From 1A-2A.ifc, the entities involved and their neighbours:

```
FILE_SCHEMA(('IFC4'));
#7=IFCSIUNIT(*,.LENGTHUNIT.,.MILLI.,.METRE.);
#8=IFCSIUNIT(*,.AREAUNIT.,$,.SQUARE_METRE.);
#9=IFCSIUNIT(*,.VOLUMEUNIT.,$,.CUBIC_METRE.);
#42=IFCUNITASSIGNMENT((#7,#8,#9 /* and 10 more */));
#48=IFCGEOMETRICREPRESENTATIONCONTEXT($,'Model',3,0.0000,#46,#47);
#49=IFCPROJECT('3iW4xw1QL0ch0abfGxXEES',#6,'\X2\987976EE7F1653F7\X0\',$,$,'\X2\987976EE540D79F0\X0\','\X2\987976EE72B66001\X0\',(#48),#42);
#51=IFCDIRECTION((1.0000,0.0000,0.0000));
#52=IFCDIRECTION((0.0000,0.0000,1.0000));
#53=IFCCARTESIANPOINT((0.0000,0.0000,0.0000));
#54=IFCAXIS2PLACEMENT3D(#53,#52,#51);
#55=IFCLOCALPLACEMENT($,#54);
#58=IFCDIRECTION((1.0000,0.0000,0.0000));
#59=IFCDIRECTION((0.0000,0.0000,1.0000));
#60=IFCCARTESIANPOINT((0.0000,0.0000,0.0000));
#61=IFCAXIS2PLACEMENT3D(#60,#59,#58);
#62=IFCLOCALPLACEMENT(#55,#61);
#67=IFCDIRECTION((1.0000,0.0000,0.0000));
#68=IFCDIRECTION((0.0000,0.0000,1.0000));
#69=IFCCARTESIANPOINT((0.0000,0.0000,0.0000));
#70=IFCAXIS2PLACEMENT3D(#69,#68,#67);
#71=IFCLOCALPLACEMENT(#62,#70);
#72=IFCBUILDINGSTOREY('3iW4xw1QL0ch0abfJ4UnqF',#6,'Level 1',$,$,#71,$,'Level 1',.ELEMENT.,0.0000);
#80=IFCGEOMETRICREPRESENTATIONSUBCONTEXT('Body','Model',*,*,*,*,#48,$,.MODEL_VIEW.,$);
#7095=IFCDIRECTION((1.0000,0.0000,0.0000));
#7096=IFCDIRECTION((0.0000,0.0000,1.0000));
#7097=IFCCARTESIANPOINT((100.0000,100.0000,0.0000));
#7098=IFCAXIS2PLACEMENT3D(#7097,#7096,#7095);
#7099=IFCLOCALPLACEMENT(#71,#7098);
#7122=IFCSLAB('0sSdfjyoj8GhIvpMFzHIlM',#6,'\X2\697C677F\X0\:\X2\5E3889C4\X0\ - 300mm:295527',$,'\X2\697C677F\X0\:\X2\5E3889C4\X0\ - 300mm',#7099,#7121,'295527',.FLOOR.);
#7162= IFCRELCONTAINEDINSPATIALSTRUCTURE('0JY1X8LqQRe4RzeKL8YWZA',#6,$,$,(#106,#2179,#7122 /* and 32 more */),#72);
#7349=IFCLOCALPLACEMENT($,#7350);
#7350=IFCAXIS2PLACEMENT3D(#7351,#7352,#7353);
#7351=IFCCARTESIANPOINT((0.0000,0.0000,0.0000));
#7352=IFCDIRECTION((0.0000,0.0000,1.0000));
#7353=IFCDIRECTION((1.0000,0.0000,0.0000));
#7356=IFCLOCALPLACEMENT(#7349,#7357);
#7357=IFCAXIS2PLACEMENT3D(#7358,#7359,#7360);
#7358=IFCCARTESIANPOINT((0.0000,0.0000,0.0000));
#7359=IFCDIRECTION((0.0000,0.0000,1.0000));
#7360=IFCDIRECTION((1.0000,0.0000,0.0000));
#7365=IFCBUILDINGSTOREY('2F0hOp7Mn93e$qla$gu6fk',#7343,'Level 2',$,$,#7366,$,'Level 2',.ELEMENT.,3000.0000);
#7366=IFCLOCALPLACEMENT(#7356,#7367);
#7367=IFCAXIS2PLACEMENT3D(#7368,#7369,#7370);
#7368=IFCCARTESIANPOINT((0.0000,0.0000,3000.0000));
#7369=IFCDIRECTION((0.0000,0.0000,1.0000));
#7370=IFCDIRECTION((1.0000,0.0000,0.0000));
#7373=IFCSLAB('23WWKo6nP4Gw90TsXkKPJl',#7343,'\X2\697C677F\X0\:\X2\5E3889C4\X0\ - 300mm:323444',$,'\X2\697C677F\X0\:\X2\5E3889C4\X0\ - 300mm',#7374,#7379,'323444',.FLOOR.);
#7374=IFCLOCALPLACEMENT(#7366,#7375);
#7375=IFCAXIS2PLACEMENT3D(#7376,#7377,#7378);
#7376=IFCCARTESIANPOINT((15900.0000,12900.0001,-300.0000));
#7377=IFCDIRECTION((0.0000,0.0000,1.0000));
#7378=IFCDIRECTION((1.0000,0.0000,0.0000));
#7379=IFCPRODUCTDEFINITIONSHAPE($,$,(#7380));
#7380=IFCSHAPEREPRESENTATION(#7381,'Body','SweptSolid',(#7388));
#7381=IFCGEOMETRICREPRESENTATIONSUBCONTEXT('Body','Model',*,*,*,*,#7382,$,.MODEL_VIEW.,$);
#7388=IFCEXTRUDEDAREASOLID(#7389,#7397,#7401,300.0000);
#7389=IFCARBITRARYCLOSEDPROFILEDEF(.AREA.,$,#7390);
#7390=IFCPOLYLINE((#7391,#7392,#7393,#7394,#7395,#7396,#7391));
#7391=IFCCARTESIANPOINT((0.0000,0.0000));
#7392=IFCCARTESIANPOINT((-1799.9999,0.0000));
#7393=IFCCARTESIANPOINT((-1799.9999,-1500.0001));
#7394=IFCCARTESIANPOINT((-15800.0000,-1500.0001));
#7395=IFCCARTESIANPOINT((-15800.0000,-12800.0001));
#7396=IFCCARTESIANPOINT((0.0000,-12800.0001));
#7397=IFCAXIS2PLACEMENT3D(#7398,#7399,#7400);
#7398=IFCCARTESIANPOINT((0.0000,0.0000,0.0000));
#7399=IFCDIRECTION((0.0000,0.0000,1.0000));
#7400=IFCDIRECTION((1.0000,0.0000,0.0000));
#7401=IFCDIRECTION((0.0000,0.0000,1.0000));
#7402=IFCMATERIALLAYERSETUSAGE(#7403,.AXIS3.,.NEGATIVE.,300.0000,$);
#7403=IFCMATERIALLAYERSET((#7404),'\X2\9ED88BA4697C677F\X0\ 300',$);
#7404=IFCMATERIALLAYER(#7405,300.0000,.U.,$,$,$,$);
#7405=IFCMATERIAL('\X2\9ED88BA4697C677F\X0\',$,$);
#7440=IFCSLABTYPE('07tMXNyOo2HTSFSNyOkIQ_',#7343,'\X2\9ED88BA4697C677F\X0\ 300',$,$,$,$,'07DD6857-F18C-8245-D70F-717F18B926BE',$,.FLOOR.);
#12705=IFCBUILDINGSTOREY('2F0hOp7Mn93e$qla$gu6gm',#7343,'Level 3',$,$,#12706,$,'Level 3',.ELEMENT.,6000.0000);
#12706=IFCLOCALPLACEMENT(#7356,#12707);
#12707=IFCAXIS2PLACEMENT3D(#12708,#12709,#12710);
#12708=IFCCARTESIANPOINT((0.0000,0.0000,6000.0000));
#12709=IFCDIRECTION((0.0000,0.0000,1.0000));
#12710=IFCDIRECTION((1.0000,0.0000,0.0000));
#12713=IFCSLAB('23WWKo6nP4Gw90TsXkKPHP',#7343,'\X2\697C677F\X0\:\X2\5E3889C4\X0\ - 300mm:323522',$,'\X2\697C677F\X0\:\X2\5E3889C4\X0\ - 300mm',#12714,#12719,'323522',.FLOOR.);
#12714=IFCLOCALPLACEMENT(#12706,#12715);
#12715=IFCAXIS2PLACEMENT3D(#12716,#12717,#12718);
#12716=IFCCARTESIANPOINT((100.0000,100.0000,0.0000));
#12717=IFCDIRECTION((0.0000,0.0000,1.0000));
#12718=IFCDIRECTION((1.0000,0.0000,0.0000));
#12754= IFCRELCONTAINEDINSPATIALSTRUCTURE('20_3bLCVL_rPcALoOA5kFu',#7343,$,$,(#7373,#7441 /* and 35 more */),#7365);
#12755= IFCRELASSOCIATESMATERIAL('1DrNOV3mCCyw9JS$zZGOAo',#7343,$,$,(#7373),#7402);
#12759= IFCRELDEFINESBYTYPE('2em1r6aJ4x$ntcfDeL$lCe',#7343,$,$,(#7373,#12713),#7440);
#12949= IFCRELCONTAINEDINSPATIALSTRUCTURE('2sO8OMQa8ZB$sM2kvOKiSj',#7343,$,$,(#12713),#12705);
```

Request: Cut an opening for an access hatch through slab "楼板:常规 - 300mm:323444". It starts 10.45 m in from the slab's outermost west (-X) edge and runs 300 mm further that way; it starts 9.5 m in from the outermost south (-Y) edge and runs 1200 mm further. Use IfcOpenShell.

```python
import numpy as np
import ifcopenshell
import ifcopenshell.api.feature
import ifcopenshell.api.geometry
import ifcopenshell.api.root
import ifcopenshell.geom
import ifcopenshell.util.placement
import ifcopenshell.util.representation
import ifcopenshell.util.shape
import ifcopenshell.util.unit

model = ifcopenshell.open("1A-2A.ifc")
unit_scale = ifcopenshell.util.unit.calculate_unit_scale(model)
settings = ifcopenshell.geom.settings()


def volume(element):
    """Net volume in cubic metres, openings subtracted."""
    shape = ifcopenshell.geom.create_shape(settings, element)
    return ifcopenshell.util.shape.get_volume(shape.geometry)


slab = model.by_guid("23WWKo6nP4Gw90TsXkKPJl")
before = volume(slab)

# Extent in the slab's own axes, in metres. The edges named are its -X and -Y sides.
slab_shape = ifcopenshell.geom.create_shape(settings, slab)
vertices = ifcopenshell.util.shape.get_vertices(slab_shape.geometry)
x_min, y_min, bottom = vertices.min(axis=0)
top = vertices[:, 2].max()

opening = ifcopenshell.api.root.create_entity(model, ifc_class="IfcOpeningElement", name="Access hatch opening", predefined_type="OPENING")
context = ifcopenshell.util.representation.get_context(model, "Model", "Body", "MODEL_VIEW")
width, depth = 0.3, 1.2
outline = [(0.0, 0.0), (width, 0.0), (width, depth), (0.0, depth), (0.0, 0.0)]
# Overshoot both faces by 50 mm so the cut is clean.
shape = ifcopenshell.api.geometry.add_slab_representation(
    model, context=context, depth=top - bottom + 0.1, polyline=outline
)
ifcopenshell.api.geometry.assign_representation(model, product=opening, representation=shape)

matrix = ifcopenshell.util.placement.get_local_placement(slab.ObjectPlacement)
matrix[:, 3] = matrix @ np.append(np.array([x_min + 10.45, y_min + 9.5, bottom - 0.05]) / unit_scale, 1.0)
ifcopenshell.api.geometry.edit_object_placement(model, product=opening, matrix=matrix, is_si=False)
ifcopenshell.api.feature.add_feature(model, feature=opening, element=slab)

after = volume(slab)

print(f"slab volume {before:.3f} -> {after:.3f} m3")

model.write("1A-2A_v2.ifc")
```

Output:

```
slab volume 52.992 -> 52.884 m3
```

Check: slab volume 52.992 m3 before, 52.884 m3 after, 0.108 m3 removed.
